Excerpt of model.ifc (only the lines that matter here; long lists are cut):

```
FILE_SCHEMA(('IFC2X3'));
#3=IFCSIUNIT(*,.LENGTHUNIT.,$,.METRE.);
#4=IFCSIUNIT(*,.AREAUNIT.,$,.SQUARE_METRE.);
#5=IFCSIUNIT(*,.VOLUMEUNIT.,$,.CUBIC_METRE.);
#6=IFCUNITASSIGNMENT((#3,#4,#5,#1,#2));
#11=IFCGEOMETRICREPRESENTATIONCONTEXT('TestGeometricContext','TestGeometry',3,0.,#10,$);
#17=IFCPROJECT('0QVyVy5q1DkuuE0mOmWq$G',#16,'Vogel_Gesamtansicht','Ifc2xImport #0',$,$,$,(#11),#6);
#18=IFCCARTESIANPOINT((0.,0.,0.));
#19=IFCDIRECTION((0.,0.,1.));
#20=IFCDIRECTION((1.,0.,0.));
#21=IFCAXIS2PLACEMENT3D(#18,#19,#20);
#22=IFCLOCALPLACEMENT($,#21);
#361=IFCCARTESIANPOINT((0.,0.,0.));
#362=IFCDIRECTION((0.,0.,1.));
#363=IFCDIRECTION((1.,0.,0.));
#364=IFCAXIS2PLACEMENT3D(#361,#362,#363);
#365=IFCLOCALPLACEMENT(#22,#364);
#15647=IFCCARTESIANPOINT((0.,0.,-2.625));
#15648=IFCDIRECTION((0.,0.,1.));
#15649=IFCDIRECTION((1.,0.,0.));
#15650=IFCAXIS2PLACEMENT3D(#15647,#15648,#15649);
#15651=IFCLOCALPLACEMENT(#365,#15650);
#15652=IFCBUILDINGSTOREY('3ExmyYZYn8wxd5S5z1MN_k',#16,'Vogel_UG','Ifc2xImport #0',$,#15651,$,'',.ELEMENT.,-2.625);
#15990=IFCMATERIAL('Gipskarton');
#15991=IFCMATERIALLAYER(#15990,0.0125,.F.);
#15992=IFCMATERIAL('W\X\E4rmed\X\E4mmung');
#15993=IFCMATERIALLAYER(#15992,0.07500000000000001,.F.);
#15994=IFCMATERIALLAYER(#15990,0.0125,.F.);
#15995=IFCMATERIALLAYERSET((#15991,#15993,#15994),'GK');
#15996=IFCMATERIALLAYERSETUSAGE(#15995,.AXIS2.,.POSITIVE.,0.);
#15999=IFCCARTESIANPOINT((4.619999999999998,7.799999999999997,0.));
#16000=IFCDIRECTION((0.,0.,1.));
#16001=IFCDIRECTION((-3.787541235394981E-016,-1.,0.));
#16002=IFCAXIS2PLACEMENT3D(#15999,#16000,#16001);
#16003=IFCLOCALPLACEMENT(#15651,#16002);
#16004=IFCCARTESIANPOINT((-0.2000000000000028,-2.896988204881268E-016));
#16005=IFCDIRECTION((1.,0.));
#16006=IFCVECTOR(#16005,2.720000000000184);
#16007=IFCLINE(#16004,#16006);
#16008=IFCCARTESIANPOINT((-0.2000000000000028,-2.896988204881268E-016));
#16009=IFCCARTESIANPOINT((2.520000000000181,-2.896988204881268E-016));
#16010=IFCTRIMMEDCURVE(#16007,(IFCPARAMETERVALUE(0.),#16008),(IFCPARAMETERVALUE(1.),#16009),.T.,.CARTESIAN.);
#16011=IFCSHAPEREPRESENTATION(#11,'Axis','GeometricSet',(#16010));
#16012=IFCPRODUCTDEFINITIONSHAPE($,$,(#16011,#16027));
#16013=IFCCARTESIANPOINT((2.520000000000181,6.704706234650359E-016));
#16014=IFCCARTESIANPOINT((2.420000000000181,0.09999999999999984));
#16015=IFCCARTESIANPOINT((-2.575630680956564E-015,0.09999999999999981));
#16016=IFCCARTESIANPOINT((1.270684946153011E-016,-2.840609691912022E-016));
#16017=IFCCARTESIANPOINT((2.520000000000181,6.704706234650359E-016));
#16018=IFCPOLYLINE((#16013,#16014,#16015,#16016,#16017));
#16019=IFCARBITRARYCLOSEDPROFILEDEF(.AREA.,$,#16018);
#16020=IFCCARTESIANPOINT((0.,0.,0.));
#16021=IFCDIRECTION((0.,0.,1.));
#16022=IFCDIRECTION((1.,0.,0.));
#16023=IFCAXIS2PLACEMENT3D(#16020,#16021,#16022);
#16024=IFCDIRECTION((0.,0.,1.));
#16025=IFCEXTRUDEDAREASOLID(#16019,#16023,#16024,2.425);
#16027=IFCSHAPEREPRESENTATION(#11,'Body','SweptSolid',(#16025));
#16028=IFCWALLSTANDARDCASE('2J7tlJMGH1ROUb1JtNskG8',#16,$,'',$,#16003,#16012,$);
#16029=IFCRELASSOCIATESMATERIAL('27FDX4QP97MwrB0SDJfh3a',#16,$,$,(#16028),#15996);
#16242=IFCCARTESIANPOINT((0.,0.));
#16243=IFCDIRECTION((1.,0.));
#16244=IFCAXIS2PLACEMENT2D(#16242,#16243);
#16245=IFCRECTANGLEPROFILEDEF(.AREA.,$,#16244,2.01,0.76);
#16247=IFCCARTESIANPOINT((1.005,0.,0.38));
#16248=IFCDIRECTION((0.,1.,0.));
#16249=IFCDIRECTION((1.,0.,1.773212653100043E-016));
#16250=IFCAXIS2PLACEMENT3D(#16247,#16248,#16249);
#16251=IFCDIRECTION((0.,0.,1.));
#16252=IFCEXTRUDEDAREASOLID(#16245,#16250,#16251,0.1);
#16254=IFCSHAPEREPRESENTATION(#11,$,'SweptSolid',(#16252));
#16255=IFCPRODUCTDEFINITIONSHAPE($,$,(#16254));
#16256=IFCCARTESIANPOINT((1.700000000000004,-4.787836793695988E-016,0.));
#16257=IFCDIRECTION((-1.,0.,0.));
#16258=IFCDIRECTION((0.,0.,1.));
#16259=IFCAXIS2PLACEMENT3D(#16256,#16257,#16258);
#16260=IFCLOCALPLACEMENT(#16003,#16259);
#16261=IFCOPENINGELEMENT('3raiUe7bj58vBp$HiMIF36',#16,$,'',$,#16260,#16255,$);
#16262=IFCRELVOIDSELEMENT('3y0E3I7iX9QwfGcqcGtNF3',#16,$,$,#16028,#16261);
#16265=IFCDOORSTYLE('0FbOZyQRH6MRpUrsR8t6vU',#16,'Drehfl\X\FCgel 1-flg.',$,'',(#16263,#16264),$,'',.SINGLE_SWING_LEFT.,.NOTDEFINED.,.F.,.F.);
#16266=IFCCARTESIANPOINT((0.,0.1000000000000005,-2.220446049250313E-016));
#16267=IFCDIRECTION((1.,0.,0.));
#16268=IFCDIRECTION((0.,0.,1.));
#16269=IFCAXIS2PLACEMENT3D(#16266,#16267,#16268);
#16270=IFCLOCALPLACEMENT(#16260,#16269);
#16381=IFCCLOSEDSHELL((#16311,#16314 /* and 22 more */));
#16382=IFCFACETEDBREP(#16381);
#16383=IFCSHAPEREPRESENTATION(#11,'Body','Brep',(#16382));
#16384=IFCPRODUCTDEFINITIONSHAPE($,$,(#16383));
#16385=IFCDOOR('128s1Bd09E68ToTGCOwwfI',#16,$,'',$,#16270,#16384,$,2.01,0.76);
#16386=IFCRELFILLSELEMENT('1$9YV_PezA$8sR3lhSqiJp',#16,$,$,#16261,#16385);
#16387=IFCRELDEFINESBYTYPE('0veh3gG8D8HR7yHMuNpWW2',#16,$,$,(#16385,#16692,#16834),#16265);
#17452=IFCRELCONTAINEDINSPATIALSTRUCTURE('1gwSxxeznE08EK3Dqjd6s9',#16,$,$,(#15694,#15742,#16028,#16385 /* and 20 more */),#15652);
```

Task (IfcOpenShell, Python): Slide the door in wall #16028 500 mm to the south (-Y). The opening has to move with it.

```python
import ifcopenshell
import ifcopenshell.api.geometry
import ifcopenshell.util.placement

model = ifcopenshell.open("model.ifc")

door = model.by_id(16385)
opening = door.FillsVoids[0].RelatingOpeningElement
wall = opening.VoidsElements[0].RelatingBuildingElement

wall_matrix = ifcopenshell.util.placement.get_local_placement(wall.ObjectPlacement)
shift = wall_matrix[:3, 0] * 0.5
before = ifcopenshell.util.placement.get_local_placement(door.ObjectPlacement)[:3, 3].copy()

# The door is placed relative to its opening, so it follows when the opening moves.
matrix = ifcopenshell.util.placement.get_local_placement(opening.ObjectPlacement)
matrix[:3, 3] += shift
ifcopenshell.api.geometry.edit_object_placement(
    model, product=opening, matrix=matrix, is_si=False, should_transform_children=True
)

after = ifcopenshell.util.placement.get_local_placement(door.ObjectPlacement)[:3, 3]
print("door moved by", (after - before).round(3) + 0.0)

model.write("model_edited.ifc")
```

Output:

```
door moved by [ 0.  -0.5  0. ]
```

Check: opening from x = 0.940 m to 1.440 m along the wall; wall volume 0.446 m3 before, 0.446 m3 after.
